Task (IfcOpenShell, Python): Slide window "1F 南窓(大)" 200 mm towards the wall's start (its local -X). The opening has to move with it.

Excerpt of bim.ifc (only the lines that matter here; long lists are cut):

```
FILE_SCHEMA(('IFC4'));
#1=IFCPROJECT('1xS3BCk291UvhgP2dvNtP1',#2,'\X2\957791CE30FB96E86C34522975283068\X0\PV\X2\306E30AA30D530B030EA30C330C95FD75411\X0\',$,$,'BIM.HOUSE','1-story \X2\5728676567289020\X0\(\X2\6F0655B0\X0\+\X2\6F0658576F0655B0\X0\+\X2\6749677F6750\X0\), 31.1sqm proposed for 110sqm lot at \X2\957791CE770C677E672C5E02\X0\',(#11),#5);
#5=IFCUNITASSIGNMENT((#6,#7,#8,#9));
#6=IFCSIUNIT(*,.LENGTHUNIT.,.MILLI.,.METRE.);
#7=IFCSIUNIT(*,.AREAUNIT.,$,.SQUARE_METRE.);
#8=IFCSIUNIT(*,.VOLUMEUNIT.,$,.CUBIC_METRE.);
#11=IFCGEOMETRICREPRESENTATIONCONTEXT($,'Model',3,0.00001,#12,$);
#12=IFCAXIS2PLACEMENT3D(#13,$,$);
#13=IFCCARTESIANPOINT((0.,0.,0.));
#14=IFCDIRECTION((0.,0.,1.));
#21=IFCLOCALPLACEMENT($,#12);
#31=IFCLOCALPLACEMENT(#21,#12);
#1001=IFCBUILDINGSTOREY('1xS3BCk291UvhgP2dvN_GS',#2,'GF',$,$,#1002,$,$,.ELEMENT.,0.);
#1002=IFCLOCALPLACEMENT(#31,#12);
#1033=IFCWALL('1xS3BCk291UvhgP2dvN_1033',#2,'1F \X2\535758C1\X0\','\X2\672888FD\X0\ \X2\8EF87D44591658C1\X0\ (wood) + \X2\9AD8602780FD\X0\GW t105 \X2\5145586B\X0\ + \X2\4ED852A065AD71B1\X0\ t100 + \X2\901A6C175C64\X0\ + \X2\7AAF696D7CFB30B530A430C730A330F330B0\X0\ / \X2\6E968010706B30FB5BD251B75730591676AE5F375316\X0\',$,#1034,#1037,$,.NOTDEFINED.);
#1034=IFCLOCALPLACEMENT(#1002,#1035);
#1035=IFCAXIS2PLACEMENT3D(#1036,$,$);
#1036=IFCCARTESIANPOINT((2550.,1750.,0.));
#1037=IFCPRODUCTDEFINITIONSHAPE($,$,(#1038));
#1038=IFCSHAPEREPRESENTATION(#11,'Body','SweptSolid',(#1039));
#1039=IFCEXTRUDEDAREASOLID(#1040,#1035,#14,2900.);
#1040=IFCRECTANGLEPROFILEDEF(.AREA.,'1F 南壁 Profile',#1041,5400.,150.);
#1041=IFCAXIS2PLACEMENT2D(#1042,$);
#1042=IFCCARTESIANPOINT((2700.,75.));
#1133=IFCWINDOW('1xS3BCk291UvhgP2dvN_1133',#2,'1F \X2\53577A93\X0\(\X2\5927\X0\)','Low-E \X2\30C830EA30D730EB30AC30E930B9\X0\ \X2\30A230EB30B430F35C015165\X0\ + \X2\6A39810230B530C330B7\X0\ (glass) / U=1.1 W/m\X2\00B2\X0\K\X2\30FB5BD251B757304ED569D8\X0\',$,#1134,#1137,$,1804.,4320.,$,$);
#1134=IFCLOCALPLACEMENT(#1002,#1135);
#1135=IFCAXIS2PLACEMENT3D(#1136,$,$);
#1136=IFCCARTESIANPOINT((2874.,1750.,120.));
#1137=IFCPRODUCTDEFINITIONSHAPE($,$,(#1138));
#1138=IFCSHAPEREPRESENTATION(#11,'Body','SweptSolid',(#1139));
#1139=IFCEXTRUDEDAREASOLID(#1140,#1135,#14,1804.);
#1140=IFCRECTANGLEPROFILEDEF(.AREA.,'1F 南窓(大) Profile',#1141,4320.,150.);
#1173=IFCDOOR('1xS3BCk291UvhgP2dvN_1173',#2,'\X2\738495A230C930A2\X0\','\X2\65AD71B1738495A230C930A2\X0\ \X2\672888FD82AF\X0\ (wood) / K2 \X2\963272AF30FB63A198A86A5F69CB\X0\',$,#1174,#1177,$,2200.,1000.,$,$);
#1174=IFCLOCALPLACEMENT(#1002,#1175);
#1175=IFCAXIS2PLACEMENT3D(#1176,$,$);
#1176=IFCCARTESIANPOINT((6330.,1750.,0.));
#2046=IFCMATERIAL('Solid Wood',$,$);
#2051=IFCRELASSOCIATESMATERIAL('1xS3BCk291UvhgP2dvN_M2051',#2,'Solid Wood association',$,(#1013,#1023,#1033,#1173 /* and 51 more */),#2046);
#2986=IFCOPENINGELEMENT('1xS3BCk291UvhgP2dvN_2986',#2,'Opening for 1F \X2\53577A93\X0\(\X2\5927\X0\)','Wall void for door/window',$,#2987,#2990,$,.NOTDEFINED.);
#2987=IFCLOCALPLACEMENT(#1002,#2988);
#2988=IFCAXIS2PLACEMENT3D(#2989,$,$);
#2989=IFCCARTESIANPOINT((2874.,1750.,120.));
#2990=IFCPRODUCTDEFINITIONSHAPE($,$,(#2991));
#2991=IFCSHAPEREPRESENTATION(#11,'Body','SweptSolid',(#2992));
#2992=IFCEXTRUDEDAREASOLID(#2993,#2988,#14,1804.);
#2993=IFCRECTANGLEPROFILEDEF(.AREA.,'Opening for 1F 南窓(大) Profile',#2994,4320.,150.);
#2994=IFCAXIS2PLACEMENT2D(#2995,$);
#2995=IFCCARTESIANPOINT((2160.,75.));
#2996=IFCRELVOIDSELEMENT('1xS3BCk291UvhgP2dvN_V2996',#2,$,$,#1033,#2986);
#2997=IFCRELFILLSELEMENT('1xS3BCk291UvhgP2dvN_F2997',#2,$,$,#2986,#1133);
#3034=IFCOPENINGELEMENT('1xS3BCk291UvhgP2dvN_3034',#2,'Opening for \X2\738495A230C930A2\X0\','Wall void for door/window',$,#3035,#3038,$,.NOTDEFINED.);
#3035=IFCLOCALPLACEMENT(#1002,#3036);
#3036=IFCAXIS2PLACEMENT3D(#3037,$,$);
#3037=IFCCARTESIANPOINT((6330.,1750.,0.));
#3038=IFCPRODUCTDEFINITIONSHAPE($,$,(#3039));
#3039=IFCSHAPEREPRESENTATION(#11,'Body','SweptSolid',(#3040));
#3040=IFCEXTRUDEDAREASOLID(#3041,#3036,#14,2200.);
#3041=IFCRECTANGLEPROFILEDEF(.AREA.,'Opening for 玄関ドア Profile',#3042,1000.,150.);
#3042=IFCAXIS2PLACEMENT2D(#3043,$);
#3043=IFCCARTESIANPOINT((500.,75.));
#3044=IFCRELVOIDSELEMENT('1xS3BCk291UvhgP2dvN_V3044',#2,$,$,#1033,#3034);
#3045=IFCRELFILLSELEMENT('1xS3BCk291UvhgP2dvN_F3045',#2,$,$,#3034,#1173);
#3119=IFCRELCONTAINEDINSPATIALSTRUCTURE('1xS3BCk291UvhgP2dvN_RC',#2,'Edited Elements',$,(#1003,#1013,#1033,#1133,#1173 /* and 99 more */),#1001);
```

```python
import ifcopenshell
import ifcopenshell.api.geometry
import ifcopenshell.util.placement

model = ifcopenshell.open("bim.ifc")

window = model.by_guid("1xS3BCk291UvhgP2dvN_1133")
opening = window.FillsVoids[0].RelatingOpeningElement
wall = opening.VoidsElements[0].RelatingBuildingElement

wall_matrix = ifcopenshell.util.placement.get_local_placement(wall.ObjectPlacement)
shift = wall_matrix[:3, 0] * -200.0
before = ifcopenshell.util.placement.get_local_placement(window.ObjectPlacement)[:3, 3].copy()

# The window is not placed relative to its opening, so move both.
for product in (opening, window):
    matrix = ifcopenshell.util.placement.get_local_placement(product.ObjectPlacement)
    matrix[:3, 3] += shift
    ifcopenshell.api.geometry.edit_object_placement(model, product=product, matrix=matrix, is_si=False)

after = ifcopenshell.util.placement.get_local_placement(window.ObjectPlacement)[:3, 3]
print("window moved by", (after - before).round(3) + 0.0)

model.write("bim-out.ifc")
```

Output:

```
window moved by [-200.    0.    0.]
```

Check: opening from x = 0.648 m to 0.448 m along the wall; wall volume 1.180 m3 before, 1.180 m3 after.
